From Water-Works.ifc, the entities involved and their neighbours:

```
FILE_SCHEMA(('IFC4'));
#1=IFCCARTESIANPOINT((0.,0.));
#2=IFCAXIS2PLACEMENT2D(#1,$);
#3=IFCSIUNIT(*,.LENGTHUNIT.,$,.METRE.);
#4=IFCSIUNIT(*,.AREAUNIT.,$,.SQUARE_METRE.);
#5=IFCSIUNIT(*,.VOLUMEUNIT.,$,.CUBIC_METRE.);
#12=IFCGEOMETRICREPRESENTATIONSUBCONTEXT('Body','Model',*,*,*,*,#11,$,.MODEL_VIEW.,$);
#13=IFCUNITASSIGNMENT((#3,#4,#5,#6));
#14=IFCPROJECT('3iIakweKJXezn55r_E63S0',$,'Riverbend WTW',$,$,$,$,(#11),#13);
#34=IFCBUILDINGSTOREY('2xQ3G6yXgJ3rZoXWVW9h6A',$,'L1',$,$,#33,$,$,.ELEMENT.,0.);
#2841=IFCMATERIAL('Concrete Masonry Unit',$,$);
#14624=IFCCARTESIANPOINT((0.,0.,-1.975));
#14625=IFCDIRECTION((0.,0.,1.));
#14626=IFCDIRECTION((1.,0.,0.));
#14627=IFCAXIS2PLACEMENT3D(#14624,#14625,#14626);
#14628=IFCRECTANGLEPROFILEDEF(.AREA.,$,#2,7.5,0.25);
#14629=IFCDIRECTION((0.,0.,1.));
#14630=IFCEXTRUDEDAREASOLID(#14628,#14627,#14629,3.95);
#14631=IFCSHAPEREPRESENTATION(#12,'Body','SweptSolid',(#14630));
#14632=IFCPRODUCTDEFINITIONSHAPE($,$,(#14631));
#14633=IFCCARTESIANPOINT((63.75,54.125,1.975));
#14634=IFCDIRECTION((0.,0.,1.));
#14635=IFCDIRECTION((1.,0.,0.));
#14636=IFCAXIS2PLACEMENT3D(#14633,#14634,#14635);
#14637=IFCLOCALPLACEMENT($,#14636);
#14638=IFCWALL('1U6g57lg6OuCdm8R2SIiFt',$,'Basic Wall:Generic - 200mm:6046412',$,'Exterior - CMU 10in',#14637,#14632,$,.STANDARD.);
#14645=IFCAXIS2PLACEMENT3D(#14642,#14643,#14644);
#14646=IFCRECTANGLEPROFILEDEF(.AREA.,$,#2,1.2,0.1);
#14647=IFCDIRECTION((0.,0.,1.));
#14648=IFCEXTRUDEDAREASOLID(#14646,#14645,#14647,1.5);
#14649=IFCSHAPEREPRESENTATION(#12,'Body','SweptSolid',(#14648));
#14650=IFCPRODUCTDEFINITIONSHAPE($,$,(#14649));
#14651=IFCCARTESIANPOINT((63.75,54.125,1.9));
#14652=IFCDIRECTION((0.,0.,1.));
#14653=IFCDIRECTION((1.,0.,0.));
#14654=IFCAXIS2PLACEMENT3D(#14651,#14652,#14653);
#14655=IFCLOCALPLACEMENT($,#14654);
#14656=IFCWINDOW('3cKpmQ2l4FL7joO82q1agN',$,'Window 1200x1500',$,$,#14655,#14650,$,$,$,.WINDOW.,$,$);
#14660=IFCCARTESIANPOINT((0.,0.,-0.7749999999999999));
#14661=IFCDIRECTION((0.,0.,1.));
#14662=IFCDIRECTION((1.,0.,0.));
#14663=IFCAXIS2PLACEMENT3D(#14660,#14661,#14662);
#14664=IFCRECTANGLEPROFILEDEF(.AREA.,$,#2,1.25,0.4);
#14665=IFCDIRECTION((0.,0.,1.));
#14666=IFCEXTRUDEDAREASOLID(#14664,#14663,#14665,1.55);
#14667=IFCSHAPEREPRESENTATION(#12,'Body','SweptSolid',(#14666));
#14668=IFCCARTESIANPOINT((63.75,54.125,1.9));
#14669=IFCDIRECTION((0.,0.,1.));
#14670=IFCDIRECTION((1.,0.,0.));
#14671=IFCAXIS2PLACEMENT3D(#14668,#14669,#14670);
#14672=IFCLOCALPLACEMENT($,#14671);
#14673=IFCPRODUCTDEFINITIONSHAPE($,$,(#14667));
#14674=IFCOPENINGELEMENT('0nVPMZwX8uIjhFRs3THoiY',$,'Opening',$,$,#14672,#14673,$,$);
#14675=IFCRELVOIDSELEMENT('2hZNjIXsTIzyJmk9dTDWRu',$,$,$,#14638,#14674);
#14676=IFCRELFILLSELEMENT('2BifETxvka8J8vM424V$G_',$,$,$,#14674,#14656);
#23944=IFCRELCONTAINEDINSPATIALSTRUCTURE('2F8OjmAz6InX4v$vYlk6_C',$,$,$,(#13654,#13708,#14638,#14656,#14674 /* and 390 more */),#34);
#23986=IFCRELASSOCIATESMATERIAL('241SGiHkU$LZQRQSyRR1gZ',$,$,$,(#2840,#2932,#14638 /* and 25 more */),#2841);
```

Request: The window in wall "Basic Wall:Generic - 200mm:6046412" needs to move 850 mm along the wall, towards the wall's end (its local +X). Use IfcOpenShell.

```python
import ifcopenshell
import ifcopenshell.api.geometry
import ifcopenshell.util.placement
import ifcopenshell.util.unit

model = ifcopenshell.open("Water-Works.ifc")
unit_scale = ifcopenshell.util.unit.calculate_unit_scale(model)

window = model.by_guid("3cKpmQ2l4FL7joO82q1agN")
opening = window.FillsVoids[0].RelatingOpeningElement
wall = opening.VoidsElements[0].RelatingBuildingElement

wall_matrix = ifcopenshell.util.placement.get_local_placement(wall.ObjectPlacement)
shift = wall_matrix[:3, 0] * 0.85 / unit_scale
before = ifcopenshell.util.placement.get_local_placement(window.ObjectPlacement)[:3, 3].copy()

# The window is not placed relative to its opening, so move both.
for product in (opening, window):
    matrix = ifcopenshell.util.placement.get_local_placement(product.ObjectPlacement)
    matrix[:3, 3] += shift
    ifcopenshell.api.geometry.edit_object_placement(model, product=product, matrix=matrix, is_si=False)

after = ifcopenshell.util.placement.get_local_placement(window.ObjectPlacement)[:3, 3]
print("window moved by", (after - before).round(3) + 0.0)

model.write("Water-Works_updated.ifc")
```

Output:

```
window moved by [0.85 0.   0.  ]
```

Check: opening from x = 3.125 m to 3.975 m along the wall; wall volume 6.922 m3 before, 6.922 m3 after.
